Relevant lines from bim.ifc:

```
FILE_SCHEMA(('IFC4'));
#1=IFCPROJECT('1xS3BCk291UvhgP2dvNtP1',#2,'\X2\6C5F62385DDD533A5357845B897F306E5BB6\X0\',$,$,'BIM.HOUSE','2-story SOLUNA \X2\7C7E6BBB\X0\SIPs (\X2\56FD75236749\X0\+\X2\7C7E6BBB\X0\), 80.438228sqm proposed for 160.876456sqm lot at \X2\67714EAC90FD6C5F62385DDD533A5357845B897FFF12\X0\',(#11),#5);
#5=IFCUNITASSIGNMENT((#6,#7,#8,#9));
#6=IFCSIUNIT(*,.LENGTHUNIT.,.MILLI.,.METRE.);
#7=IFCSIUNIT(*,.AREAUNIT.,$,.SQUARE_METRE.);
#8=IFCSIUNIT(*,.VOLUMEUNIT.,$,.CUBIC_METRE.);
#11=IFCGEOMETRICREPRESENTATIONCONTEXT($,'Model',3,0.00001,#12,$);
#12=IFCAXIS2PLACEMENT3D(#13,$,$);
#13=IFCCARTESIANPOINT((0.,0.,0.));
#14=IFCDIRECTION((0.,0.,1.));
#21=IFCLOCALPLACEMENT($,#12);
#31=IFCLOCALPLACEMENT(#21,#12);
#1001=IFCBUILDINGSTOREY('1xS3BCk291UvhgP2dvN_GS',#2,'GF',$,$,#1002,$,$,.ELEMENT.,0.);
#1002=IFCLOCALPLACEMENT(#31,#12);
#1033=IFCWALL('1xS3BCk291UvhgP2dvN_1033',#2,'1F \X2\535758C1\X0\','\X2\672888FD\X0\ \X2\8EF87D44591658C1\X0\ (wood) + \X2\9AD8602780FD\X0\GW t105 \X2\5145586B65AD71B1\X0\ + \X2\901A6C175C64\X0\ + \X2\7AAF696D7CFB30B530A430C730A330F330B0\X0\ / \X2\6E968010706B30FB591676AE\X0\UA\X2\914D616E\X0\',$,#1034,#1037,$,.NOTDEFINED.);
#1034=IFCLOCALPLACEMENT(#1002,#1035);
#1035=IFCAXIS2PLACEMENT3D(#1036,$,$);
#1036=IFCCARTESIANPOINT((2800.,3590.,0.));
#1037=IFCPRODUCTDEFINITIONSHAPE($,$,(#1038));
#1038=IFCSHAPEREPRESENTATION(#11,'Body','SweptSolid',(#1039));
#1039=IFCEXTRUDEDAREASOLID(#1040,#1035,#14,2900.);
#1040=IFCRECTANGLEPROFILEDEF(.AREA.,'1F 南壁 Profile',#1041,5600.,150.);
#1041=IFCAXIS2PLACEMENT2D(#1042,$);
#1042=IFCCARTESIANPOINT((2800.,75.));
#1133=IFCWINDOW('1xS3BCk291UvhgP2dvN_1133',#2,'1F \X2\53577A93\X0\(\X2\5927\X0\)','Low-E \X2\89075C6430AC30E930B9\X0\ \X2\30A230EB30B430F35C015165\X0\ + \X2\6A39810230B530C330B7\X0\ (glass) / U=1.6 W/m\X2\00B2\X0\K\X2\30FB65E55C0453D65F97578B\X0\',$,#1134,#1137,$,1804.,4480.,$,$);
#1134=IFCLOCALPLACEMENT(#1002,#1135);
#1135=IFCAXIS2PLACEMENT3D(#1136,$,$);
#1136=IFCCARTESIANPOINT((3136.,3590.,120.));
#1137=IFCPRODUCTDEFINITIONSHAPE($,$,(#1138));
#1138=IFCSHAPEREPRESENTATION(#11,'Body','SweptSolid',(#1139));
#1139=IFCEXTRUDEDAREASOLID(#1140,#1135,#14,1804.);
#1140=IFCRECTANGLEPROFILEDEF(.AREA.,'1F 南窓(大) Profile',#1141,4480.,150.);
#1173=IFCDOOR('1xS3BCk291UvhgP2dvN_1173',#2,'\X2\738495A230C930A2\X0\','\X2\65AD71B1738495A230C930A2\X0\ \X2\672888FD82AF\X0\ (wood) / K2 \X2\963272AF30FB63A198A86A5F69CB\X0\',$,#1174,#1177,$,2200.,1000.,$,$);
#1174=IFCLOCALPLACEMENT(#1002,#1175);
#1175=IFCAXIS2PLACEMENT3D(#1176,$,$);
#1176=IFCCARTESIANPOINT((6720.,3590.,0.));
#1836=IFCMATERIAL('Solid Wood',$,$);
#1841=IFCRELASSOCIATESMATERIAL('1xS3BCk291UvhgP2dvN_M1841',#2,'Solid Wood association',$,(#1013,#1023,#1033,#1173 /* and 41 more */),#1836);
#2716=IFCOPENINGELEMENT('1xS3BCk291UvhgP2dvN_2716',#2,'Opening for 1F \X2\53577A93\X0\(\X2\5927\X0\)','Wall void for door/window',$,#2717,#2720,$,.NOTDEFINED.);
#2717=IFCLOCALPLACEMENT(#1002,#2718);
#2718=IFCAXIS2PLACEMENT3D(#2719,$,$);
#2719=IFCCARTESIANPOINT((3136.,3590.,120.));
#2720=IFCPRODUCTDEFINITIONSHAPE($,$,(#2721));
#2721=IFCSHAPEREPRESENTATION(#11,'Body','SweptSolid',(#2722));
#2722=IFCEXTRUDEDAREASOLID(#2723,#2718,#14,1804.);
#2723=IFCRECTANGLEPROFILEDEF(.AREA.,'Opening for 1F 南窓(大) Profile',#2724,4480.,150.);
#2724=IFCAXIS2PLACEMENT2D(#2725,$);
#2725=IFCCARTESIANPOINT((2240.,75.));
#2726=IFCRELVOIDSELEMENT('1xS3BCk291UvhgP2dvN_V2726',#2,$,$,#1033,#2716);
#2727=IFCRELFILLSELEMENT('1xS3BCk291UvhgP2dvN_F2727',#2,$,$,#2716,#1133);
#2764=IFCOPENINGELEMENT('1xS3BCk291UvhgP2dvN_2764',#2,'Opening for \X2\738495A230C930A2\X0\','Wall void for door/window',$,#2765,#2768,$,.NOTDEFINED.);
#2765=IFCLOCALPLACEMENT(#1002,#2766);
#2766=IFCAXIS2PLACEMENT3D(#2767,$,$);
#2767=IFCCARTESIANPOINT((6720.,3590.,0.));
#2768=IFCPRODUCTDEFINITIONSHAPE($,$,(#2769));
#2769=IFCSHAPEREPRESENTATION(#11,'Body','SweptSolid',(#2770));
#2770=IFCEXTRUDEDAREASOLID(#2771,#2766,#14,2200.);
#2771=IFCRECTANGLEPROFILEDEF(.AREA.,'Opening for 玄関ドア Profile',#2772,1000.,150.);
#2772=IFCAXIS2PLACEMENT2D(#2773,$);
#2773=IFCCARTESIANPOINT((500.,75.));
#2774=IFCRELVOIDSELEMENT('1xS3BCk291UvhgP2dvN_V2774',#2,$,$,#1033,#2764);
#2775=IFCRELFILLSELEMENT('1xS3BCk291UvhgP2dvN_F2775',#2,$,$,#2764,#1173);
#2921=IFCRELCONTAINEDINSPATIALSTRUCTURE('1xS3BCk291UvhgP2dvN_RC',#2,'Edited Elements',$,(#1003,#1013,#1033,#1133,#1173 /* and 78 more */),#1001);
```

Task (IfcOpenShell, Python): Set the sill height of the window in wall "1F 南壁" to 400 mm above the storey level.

```python
import numpy as np
import ifcopenshell
import ifcopenshell.api.geometry
import ifcopenshell.geom
import ifcopenshell.util.element
import ifcopenshell.util.placement
import ifcopenshell.util.shape
import ifcopenshell.util.unit

model = ifcopenshell.open("bim.ifc")
unit_scale = ifcopenshell.util.unit.calculate_unit_scale(model)

window = model.by_guid("1xS3BCk291UvhgP2dvN_1133")
opening = window.FillsVoids[0].RelatingOpeningElement
storey = ifcopenshell.util.element.get_container(window, ifc_class="IfcBuildingStorey")
level = ifcopenshell.util.placement.get_local_placement(storey.ObjectPlacement)[2, 3]

# The opening's origin need not be at the sill, so measure its lowest point.
shape = ifcopenshell.geom.create_shape(ifcopenshell.geom.settings(), opening)
bottom = ifcopenshell.util.shape.get_shape_bottom_elevation(shape, shape.geometry) / unit_scale
dz = level + 400.0 - bottom

shift = np.array([0.0, 0.0, dz])
# The window is not placed relative to its opening, so move both.
for product in (opening, window):
    matrix = ifcopenshell.util.placement.get_local_placement(product.ObjectPlacement)
    matrix[:3, 3] += shift
    ifcopenshell.api.geometry.edit_object_placement(model, product=product, matrix=matrix, is_si=False)

print(f"moved by {dz * unit_scale:+.3f} m")

model.write("bim_v2.ifc")
```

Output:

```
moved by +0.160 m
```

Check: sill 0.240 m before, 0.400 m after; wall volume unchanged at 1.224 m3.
